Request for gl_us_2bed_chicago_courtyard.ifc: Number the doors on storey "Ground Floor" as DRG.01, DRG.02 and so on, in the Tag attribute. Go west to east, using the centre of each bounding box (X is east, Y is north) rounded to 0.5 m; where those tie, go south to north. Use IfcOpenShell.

First a look at what the model holds.

```python
import ifcopenshell
import ifcopenshell.util.element
import ifcopenshell.util.placement

model = ifcopenshell.open("gl_us_2bed_chicago_courtyard.ifc")
print(model.schema)
storey = next(s for s in model.by_type("IfcBuildingStorey") if s.Name == "Ground Floor")
doors = [e for e in ifcopenshell.util.element.get_decomposition(storey) if e.is_a("IfcDoor")]
for e in sorted(doors, key=lambda e: e.id()):
    origin = ifcopenshell.util.placement.get_local_placement(e.ObjectPlacement)[:3, 3]
    print(e.id(), e.Tag, e.Name, origin.round(2) + 0.0, sep=" | ")
```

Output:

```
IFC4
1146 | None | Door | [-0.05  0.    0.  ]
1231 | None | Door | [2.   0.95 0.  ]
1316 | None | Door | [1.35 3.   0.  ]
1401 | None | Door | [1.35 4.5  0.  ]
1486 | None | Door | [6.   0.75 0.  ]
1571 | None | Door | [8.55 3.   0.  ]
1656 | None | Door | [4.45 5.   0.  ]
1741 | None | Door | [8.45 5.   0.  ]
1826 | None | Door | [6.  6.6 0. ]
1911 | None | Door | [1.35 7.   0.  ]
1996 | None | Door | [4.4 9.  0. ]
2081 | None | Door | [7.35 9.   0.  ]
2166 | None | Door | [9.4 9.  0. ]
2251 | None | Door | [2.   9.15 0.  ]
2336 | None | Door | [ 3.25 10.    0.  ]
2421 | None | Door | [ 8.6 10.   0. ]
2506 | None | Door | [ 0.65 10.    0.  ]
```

```python
import ifcopenshell
import ifcopenshell.geom
import ifcopenshell.util.element
import ifcopenshell.util.shape

model = ifcopenshell.open("gl_us_2bed_chicago_courtyard.ifc")
settings = ifcopenshell.geom.settings()
settings.set("use-world-coords", True)


def centre(element):
    shape = ifcopenshell.geom.create_shape(settings, element)
    return ifcopenshell.util.shape.get_bbox_centroid(shape.geometry)


storey = next(s for s in model.by_type("IfcBuildingStorey") if s.Name == "Ground Floor")
doors = [e for e in ifcopenshell.util.element.get_decomposition(storey) if e.is_a("IfcDoor")]

# Insertion points can sit at a corner or the storey origin, so sort by the geometry (in metres).
centres = {e: centre(e) for e in doors}
doors.sort(key=lambda e: (round(centres[e][0] / 0.5), centres[e][1]))

for i, e in enumerate(doors, start=1):
    number = f"DRG.{i:02d}"
    e.Tag = number
    print(e.id(), number)

model.write("gl_us_2bed_chicago_courtyard_rev.ifc")
```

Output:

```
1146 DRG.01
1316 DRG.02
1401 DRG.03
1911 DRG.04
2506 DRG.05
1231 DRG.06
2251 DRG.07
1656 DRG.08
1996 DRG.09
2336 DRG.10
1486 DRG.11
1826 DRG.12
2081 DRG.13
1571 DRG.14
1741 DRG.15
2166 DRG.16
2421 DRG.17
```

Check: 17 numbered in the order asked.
